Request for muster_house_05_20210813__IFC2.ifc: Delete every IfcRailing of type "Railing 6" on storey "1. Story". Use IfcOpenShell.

First a look at what the model holds.

```python
import ifcopenshell
import ifcopenshell.util.element

model = ifcopenshell.open("muster_house_05_20210813__IFC2.ifc")
print(model.schema)
storey = next(s for s in model.by_type("IfcBuildingStorey") if s.Name == "1. Story")
railings = [e for e in ifcopenshell.util.element.get_decomposition(storey) if e.is_a("IfcRailing")]
seen = {}
for e in railings:
    element_type = ifcopenshell.util.element.get_type(e)
    name = element_type.Name if element_type not in (None, e) else None
    seen[name] = seen.get(name, 0) + 1
for name, count in sorted(seen.items(), key=str):
    print(count, "x", name)
```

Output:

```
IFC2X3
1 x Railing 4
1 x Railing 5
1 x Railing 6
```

```python
import ifcopenshell
import ifcopenshell.api.root
import ifcopenshell.util.element

model = ifcopenshell.open("muster_house_05_20210813__IFC2.ifc")

storey = next(s for s in model.by_type("IfcBuildingStorey") if s.Name == "1. Story")
railings = [e for e in ifcopenshell.util.element.get_decomposition(storey) if e.is_a("IfcRailing")]
targets = [e for e in railings if (t := ifcopenshell.util.element.get_type(e)) not in (None, e) and t.Name == "Railing 6"]

for e in targets:
    ifcopenshell.api.root.remove_product(model, product=e)
print(len(targets), "removed")

model.write("muster_house_05_20210813__IFC2_edited.ifc")
```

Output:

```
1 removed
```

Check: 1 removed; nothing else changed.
